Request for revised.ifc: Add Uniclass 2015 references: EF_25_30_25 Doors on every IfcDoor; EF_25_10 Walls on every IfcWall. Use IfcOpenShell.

First a look at what the model holds.

```python
import ifcopenshell

model = ifcopenshell.open("revised.ifc")
print(model.schema)
print("classifications:", [c.Name for c in model.by_type("IfcClassification")])
for ifc_class in ("IfcDoor", "IfcRoof", "IfcStair", "IfcWall", "IfcWindow"):
    print(ifc_class, len(model.by_type(ifc_class)))
```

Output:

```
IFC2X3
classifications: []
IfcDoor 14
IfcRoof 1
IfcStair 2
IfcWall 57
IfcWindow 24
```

```python
import ifcopenshell
import ifcopenshell.api.classification

model = ifcopenshell.open("revised.ifc")

# IFC2X3 requires Source and Edition and has no link from the project to the system.
system = model.create_entity("IfcClassification", Source="NBS", Edition="2015", Name="Uniclass 2015")

codes = {
    "IfcDoor": ("EF_25_30_25", "Doors"),
    "IfcWall": ("EF_25_10", "Walls"),
}
for ifc_class, (code, name) in codes.items():
    products = model.by_type(ifc_class)
    ifcopenshell.api.classification.add_reference(
        model, products=products, classification=system, identification=code, name=name
    )
    print(code, len(products))

model.write("revised_v2.ifc")
```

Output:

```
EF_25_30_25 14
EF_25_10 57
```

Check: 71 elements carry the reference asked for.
